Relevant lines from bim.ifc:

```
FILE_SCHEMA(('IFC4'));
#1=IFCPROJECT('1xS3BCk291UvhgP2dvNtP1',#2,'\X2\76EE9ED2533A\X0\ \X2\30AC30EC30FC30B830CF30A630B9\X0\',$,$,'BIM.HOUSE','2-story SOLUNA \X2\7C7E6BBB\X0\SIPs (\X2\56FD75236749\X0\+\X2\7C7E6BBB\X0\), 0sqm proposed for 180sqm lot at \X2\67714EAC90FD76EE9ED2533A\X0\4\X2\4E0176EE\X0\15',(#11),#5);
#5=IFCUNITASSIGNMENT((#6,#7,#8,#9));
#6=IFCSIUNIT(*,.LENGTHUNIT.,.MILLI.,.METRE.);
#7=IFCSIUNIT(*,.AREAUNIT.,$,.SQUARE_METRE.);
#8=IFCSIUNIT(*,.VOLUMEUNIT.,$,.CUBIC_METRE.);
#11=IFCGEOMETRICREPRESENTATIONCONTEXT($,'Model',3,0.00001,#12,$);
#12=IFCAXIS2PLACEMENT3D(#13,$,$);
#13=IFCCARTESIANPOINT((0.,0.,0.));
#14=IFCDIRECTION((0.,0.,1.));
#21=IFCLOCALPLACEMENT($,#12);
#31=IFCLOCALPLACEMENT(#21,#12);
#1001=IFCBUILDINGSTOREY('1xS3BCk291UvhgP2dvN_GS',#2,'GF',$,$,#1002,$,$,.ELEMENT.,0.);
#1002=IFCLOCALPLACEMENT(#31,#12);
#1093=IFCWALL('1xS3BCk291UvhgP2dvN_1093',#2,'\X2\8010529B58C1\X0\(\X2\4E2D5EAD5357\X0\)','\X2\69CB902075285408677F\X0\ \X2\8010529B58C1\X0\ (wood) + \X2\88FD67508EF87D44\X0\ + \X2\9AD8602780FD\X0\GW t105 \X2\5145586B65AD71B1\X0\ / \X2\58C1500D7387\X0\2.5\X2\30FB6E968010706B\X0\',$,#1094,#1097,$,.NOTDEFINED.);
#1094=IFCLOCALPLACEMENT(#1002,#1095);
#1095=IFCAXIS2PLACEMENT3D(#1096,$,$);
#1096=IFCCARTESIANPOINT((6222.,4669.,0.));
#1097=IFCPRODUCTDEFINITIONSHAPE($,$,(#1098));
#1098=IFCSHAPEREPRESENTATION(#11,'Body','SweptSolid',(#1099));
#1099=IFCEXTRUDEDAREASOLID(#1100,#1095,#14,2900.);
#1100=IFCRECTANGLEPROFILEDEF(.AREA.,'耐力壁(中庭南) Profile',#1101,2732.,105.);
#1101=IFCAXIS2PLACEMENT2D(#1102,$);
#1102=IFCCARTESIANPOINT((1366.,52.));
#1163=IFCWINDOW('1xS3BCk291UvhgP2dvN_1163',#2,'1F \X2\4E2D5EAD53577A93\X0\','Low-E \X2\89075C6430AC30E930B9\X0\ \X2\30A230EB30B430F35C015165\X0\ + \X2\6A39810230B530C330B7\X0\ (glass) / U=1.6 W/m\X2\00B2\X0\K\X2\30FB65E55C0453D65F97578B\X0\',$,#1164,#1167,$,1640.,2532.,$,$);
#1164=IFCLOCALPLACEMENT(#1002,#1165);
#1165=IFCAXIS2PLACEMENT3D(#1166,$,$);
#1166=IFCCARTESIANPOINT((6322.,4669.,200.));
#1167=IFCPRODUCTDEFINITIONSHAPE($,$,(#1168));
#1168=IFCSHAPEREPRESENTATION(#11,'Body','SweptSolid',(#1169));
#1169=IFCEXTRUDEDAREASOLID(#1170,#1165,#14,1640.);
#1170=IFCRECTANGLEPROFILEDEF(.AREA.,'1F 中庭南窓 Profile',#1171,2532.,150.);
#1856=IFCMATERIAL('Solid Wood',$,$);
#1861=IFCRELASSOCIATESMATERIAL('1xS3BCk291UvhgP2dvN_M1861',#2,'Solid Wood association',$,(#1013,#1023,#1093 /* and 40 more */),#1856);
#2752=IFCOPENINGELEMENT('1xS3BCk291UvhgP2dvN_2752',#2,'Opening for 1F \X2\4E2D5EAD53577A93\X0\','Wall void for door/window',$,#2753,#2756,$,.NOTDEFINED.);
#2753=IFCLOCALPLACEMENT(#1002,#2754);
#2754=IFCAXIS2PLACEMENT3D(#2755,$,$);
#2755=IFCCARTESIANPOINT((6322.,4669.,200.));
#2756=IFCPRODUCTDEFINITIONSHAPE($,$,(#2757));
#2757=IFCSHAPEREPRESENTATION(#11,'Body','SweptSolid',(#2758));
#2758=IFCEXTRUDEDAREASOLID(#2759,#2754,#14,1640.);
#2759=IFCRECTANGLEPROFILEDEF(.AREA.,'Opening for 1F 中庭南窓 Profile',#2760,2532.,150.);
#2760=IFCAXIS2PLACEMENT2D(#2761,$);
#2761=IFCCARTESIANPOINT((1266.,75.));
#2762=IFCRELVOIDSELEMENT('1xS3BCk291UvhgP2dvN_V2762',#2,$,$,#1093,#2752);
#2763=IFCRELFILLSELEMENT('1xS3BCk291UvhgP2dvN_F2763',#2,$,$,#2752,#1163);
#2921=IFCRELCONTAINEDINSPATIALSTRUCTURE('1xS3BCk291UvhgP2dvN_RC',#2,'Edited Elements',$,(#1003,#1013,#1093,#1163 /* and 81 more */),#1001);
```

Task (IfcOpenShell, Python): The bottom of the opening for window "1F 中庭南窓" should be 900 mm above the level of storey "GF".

```python
import numpy as np
import ifcopenshell
import ifcopenshell.api.geometry
import ifcopenshell.geom
import ifcopenshell.util.element
import ifcopenshell.util.placement
import ifcopenshell.util.shape
import ifcopenshell.util.unit

model = ifcopenshell.open("bim.ifc")
unit_scale = ifcopenshell.util.unit.calculate_unit_scale(model)

window = model.by_id(1163)
opening = window.FillsVoids[0].RelatingOpeningElement
storey = ifcopenshell.util.element.get_container(window, ifc_class="IfcBuildingStorey")
level = ifcopenshell.util.placement.get_local_placement(storey.ObjectPlacement)[2, 3]

# The opening's origin need not be at the sill, so measure its lowest point.
shape = ifcopenshell.geom.create_shape(ifcopenshell.geom.settings(), opening)
bottom = ifcopenshell.util.shape.get_shape_bottom_elevation(shape, shape.geometry) / unit_scale
dz = level + 0.9 / unit_scale - bottom

shift = np.array([0.0, 0.0, dz])
# The window is not placed relative to its opening, so move both.
for product in (opening, window):
    matrix = ifcopenshell.util.placement.get_local_placement(product.ObjectPlacement)
    matrix[:3, 3] += shift
    ifcopenshell.api.geometry.edit_object_placement(model, product=product, matrix=matrix, is_si=False)

print(f"moved by {dz * unit_scale:+.3f} m")

model.write("bim_rev.ifc")
```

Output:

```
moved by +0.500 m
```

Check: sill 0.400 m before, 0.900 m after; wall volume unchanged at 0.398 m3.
